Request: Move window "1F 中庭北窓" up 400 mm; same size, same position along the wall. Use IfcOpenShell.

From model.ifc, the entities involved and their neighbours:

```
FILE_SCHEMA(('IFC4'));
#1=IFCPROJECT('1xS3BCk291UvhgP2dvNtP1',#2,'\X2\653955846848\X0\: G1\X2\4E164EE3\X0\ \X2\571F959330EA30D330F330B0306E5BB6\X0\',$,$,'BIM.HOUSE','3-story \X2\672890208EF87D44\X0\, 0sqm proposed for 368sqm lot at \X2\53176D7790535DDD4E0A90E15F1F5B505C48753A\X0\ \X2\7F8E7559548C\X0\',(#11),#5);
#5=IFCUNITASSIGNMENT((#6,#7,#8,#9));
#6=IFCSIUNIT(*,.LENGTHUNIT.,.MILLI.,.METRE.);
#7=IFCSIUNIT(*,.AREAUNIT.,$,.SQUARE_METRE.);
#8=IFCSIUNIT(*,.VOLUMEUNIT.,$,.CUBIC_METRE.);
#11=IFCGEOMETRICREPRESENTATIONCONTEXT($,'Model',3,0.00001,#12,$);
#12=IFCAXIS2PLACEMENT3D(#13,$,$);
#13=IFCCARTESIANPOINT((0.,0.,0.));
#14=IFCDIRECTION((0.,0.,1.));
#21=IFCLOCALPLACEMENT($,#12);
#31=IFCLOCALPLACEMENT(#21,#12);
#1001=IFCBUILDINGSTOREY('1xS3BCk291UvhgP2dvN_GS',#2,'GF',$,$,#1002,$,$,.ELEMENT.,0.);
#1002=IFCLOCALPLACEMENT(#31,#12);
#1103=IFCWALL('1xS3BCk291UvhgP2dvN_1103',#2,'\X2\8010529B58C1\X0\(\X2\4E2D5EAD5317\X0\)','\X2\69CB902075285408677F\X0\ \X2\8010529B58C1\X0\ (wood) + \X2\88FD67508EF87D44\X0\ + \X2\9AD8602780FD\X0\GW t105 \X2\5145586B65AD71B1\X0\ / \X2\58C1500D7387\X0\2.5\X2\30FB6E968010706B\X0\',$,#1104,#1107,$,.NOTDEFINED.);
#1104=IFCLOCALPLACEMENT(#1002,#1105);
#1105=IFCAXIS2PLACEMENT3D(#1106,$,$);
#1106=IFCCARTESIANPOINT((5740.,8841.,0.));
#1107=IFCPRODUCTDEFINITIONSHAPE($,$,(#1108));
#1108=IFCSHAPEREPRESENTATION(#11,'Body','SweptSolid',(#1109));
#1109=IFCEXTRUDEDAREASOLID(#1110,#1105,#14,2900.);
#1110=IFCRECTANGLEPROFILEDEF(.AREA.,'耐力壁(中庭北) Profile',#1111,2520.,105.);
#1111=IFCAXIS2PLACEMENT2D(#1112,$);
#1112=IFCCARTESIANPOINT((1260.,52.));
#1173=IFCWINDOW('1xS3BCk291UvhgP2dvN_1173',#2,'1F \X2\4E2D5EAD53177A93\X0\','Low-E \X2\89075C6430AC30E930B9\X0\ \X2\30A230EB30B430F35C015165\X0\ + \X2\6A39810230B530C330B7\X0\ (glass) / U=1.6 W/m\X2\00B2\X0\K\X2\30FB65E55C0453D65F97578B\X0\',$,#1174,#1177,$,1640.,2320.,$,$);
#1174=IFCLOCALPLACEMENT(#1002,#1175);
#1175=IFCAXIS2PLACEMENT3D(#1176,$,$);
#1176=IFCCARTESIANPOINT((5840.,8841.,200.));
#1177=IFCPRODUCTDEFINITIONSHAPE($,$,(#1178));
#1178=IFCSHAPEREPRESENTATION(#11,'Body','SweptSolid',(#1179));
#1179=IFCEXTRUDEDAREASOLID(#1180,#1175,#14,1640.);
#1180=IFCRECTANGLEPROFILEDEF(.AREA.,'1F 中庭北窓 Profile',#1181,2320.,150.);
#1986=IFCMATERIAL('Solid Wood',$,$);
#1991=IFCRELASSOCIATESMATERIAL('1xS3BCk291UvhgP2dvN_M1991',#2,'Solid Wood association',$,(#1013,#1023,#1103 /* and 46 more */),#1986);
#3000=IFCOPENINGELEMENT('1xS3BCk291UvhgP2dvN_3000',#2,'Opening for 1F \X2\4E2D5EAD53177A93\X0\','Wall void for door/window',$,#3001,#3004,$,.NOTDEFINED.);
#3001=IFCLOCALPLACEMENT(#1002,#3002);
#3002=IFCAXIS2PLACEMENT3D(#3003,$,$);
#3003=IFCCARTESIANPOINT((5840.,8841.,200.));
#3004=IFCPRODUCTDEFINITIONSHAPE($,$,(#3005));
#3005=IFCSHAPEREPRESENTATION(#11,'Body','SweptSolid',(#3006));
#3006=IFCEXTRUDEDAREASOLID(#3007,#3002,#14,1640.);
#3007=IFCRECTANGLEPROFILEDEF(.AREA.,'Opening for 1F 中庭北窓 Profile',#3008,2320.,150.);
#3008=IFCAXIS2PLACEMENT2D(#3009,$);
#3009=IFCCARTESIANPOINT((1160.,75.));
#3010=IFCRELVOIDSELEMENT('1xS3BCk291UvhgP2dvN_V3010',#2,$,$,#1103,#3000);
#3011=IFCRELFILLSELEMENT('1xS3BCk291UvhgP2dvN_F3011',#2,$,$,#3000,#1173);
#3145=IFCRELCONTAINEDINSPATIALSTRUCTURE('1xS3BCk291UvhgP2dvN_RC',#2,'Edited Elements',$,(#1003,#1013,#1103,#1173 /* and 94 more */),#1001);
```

```python
import numpy as np
import ifcopenshell
import ifcopenshell.api.geometry
import ifcopenshell.util.placement
import ifcopenshell.util.unit

model = ifcopenshell.open("model.ifc")
unit_scale = ifcopenshell.util.unit.calculate_unit_scale(model)

window = model.by_guid("1xS3BCk291UvhgP2dvN_1173")
opening = window.FillsVoids[0].RelatingOpeningElement
dz = 0.4 / unit_scale

shift = np.array([0.0, 0.0, dz])
# The window is not placed relative to its opening, so move both.
for product in (opening, window):
    matrix = ifcopenshell.util.placement.get_local_placement(product.ObjectPlacement)
    matrix[:3, 3] += shift
    ifcopenshell.api.geometry.edit_object_placement(model, product=product, matrix=matrix, is_si=False)

print(f"moved by {dz * unit_scale:+.3f} m")

model.write("model_updated.ifc")
```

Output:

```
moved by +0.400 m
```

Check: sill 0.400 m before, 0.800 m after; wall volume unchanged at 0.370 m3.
